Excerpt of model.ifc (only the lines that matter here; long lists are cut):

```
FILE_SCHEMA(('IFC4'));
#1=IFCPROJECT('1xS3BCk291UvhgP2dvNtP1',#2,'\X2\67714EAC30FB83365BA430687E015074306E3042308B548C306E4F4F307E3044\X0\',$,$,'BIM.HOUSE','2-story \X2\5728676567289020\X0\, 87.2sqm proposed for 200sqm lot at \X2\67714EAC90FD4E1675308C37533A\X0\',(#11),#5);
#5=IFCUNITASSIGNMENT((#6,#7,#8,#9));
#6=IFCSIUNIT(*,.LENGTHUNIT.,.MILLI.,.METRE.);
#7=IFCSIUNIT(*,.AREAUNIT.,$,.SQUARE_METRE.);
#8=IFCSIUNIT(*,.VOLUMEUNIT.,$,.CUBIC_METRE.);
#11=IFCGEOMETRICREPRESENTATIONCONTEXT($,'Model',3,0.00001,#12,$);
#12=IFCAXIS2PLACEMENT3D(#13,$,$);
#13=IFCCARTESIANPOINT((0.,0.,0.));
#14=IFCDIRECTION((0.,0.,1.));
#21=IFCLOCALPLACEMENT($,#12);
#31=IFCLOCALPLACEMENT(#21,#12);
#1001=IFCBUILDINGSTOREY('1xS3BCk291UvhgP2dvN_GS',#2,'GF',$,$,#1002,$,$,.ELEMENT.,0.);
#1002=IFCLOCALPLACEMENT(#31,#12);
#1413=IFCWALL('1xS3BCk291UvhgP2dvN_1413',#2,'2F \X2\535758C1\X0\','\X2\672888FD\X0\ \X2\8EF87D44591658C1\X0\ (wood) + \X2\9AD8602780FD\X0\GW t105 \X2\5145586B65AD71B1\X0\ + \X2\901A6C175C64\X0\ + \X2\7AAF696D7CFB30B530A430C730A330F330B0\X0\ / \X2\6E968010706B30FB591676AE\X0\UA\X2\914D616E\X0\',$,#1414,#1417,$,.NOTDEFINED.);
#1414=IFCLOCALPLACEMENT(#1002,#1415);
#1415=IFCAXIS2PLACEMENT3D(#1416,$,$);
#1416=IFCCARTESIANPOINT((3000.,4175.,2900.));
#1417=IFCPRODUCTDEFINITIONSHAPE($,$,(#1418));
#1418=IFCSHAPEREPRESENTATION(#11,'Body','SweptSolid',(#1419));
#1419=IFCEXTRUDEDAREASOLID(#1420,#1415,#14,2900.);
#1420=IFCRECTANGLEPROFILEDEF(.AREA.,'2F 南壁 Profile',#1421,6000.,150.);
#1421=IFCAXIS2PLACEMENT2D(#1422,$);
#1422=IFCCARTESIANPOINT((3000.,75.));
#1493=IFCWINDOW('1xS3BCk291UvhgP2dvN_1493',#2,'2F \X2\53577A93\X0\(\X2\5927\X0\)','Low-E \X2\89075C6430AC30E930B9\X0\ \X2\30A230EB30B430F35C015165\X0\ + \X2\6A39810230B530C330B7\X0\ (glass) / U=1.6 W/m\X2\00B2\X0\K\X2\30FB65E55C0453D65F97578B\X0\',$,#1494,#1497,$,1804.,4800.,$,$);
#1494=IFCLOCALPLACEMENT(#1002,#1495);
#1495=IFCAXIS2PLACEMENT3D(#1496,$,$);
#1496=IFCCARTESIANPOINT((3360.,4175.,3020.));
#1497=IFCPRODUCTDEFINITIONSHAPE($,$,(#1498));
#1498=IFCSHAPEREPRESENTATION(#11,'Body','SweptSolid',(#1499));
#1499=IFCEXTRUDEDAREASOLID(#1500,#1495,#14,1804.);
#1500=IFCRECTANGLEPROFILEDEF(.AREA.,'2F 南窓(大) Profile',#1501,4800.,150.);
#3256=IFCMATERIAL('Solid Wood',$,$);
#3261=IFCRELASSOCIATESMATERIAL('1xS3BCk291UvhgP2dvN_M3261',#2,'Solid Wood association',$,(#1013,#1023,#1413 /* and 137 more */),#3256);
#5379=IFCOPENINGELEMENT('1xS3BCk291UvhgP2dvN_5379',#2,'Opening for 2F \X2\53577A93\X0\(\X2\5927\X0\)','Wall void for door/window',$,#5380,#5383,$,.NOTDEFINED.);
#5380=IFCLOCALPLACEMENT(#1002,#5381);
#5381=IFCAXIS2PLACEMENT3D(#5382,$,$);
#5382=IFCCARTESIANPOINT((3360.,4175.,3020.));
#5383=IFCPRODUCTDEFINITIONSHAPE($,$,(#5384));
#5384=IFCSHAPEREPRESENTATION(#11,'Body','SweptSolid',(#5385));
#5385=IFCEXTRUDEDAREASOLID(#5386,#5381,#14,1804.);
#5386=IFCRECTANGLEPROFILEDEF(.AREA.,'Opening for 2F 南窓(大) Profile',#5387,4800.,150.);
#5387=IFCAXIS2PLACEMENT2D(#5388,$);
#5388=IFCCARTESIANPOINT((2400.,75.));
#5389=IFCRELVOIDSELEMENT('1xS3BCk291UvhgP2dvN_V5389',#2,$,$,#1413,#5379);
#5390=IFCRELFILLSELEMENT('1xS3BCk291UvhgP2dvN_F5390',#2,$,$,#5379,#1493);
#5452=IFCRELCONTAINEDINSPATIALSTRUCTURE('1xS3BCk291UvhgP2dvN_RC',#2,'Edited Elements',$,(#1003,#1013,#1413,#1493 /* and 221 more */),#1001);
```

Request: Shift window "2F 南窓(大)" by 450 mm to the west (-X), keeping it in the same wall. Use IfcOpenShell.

```python
import ifcopenshell
import ifcopenshell.api.geometry
import ifcopenshell.util.placement

model = ifcopenshell.open("model.ifc")

window = model.by_id(1493)
opening = window.FillsVoids[0].RelatingOpeningElement
wall = opening.VoidsElements[0].RelatingBuildingElement

wall_matrix = ifcopenshell.util.placement.get_local_placement(wall.ObjectPlacement)
shift = wall_matrix[:3, 0] * -450.0
before = ifcopenshell.util.placement.get_local_placement(window.ObjectPlacement)[:3, 3].copy()

# The window is not placed relative to its opening, so move both.
for product in (opening, window):
    matrix = ifcopenshell.util.placement.get_local_placement(product.ObjectPlacement)
    matrix[:3, 3] += shift
    ifcopenshell.api.geometry.edit_object_placement(model, product=product, matrix=matrix, is_si=False)

after = ifcopenshell.util.placement.get_local_placement(window.ObjectPlacement)[:3, 3]
print("window moved by", (after - before).round(3) + 0.0)

model.write("model_v2.ifc")
```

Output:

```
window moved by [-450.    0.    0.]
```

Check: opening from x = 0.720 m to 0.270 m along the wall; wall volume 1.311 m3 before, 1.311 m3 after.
